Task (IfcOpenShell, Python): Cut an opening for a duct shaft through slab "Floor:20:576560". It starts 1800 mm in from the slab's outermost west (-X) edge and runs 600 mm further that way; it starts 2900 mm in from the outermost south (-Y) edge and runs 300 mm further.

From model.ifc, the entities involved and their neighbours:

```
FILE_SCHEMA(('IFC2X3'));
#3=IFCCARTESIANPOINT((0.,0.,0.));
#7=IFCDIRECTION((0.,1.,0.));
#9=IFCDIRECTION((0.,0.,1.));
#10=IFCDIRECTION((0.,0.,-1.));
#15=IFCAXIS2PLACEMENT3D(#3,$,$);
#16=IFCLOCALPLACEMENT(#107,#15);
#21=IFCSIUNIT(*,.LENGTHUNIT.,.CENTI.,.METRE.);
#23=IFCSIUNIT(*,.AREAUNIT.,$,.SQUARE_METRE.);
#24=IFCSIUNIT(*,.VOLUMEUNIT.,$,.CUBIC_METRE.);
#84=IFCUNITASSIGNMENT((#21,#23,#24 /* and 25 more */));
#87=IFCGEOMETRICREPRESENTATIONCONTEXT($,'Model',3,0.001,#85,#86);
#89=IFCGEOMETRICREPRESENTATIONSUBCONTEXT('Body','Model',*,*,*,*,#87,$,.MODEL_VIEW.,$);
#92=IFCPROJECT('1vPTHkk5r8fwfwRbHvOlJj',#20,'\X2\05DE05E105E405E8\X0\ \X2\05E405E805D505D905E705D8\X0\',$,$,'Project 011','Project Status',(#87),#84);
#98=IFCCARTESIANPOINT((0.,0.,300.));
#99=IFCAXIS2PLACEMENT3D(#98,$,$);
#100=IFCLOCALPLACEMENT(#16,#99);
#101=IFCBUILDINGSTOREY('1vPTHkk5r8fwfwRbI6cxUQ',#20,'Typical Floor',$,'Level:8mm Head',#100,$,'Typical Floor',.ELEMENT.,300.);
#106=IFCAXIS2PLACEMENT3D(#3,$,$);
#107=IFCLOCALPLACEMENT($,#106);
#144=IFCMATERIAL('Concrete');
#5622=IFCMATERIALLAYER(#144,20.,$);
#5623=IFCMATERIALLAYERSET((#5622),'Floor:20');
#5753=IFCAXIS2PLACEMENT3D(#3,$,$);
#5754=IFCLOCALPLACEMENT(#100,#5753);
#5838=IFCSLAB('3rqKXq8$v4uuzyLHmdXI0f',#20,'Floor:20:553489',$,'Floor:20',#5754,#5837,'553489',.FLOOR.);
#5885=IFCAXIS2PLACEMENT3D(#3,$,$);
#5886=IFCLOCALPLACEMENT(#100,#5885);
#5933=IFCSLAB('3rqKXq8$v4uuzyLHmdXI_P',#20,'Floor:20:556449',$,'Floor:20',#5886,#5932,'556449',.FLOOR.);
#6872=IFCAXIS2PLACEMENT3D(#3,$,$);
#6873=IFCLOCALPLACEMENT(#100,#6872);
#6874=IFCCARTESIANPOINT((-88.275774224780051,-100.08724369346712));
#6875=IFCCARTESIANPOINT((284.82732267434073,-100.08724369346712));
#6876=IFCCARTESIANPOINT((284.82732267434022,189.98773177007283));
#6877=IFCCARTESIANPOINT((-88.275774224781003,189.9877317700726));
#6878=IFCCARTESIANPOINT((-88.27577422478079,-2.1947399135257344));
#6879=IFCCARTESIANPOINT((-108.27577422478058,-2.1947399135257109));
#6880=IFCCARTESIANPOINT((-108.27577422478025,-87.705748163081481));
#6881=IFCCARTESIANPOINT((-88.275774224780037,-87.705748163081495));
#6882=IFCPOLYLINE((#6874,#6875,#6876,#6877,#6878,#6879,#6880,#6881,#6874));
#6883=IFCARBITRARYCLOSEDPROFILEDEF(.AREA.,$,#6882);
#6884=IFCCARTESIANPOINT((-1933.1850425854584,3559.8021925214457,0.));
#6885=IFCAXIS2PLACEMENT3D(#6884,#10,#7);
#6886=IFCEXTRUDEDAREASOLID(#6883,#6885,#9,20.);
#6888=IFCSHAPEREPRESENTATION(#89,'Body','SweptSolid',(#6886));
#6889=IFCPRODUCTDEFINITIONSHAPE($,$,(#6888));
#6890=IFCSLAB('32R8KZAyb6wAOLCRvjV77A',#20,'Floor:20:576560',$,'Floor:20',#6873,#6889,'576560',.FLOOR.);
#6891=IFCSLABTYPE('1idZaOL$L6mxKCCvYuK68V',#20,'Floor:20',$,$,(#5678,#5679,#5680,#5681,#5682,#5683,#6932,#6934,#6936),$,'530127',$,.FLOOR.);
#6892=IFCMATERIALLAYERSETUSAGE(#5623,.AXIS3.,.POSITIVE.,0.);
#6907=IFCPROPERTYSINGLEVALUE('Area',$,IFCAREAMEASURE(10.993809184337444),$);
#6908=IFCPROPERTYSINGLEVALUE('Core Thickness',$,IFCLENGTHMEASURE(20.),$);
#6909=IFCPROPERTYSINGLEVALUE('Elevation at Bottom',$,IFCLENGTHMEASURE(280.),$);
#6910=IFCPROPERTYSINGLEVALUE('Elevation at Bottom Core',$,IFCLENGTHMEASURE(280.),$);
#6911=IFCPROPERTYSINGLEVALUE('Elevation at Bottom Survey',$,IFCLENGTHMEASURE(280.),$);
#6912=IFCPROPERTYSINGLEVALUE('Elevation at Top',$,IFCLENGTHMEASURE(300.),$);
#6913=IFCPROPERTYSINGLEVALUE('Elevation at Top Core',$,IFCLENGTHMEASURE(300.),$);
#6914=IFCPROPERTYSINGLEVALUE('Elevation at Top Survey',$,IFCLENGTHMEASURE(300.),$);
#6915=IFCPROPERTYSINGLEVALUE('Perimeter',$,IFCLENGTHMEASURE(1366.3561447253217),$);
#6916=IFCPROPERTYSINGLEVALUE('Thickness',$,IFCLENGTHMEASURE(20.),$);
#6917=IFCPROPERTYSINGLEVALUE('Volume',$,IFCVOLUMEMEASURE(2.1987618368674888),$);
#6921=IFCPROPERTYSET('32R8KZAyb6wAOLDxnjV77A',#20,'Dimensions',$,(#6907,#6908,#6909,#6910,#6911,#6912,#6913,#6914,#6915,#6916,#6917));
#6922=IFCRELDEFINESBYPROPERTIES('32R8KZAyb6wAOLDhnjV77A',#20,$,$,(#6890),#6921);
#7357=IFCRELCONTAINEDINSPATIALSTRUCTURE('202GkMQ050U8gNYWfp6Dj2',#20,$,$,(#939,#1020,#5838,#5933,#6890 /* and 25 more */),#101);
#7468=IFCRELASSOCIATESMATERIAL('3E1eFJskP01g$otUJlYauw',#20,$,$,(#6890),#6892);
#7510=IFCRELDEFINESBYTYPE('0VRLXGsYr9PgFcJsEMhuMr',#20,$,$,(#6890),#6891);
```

```python
import numpy as np
import ifcopenshell
import ifcopenshell.api.feature
import ifcopenshell.api.geometry
import ifcopenshell.api.pset
import ifcopenshell.api.root
import ifcopenshell.geom
import ifcopenshell.util.element
import ifcopenshell.util.placement
import ifcopenshell.util.representation
import ifcopenshell.util.shape
import ifcopenshell.util.unit

model = ifcopenshell.open("model.ifc")
unit_scale = ifcopenshell.util.unit.calculate_unit_scale(model)
area_scale = ifcopenshell.util.unit.calculate_unit_scale(model, "AREAUNIT")
volume_scale = ifcopenshell.util.unit.calculate_unit_scale(model, "VOLUMEUNIT")
settings = ifcopenshell.geom.settings()


def volume(element):
    """Net volume in cubic metres, openings subtracted."""
    shape = ifcopenshell.geom.create_shape(settings, element)
    return ifcopenshell.util.shape.get_volume(shape.geometry)


slab = model.by_id(6890)
before = volume(slab)

# Extent in the slab's own axes, in metres. The edges named are its -X and -Y sides.
slab_shape = ifcopenshell.geom.create_shape(settings, slab)
vertices = ifcopenshell.util.shape.get_vertices(slab_shape.geometry)
x_min, y_min, bottom = vertices.min(axis=0)
top = vertices[:, 2].max()

opening = ifcopenshell.api.root.create_entity(model, ifc_class="IfcOpeningElement", name="Duct shaft opening")
context = ifcopenshell.util.representation.get_context(model, "Model", "Body", "MODEL_VIEW")
width, depth = 0.6, 0.3
outline = [(0.0, 0.0), (width, 0.0), (width, depth), (0.0, depth), (0.0, 0.0)]
# Overshoot both faces by 50 mm so the cut is clean.
shape = ifcopenshell.api.geometry.add_slab_representation(
    model, context=context, depth=top - bottom + 0.1, polyline=outline
)
ifcopenshell.api.geometry.assign_representation(model, product=opening, representation=shape)

matrix = ifcopenshell.util.placement.get_local_placement(slab.ObjectPlacement)
matrix[:, 3] = matrix @ np.append(np.array([x_min + 1.8, y_min + 2.9, bottom - 0.05]) / unit_scale, 1.0)
ifcopenshell.api.geometry.edit_object_placement(model, product=opening, matrix=matrix, is_si=False)
ifcopenshell.api.feature.add_feature(model, feature=opening, element=slab)

after = volume(slab)

# Update the slab's stored quantities.
pset = model.by_id(ifcopenshell.util.element.get_pset(slab, "Dimensions", should_inherit=False)["id"])
ifcopenshell.api.pset.edit_pset(model, pset=pset, properties={
    "Area": model.create_entity("IfcAreaMeasure", after / (top - bottom) / area_scale),
    "Volume": model.create_entity("IfcVolumeMeasure", after / volume_scale),
})

print(f"slab volume {before:.3f} -> {after:.3f} m3")

model.write("model_edited.ifc")
```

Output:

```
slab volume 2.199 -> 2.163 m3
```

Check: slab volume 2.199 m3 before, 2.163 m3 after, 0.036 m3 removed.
